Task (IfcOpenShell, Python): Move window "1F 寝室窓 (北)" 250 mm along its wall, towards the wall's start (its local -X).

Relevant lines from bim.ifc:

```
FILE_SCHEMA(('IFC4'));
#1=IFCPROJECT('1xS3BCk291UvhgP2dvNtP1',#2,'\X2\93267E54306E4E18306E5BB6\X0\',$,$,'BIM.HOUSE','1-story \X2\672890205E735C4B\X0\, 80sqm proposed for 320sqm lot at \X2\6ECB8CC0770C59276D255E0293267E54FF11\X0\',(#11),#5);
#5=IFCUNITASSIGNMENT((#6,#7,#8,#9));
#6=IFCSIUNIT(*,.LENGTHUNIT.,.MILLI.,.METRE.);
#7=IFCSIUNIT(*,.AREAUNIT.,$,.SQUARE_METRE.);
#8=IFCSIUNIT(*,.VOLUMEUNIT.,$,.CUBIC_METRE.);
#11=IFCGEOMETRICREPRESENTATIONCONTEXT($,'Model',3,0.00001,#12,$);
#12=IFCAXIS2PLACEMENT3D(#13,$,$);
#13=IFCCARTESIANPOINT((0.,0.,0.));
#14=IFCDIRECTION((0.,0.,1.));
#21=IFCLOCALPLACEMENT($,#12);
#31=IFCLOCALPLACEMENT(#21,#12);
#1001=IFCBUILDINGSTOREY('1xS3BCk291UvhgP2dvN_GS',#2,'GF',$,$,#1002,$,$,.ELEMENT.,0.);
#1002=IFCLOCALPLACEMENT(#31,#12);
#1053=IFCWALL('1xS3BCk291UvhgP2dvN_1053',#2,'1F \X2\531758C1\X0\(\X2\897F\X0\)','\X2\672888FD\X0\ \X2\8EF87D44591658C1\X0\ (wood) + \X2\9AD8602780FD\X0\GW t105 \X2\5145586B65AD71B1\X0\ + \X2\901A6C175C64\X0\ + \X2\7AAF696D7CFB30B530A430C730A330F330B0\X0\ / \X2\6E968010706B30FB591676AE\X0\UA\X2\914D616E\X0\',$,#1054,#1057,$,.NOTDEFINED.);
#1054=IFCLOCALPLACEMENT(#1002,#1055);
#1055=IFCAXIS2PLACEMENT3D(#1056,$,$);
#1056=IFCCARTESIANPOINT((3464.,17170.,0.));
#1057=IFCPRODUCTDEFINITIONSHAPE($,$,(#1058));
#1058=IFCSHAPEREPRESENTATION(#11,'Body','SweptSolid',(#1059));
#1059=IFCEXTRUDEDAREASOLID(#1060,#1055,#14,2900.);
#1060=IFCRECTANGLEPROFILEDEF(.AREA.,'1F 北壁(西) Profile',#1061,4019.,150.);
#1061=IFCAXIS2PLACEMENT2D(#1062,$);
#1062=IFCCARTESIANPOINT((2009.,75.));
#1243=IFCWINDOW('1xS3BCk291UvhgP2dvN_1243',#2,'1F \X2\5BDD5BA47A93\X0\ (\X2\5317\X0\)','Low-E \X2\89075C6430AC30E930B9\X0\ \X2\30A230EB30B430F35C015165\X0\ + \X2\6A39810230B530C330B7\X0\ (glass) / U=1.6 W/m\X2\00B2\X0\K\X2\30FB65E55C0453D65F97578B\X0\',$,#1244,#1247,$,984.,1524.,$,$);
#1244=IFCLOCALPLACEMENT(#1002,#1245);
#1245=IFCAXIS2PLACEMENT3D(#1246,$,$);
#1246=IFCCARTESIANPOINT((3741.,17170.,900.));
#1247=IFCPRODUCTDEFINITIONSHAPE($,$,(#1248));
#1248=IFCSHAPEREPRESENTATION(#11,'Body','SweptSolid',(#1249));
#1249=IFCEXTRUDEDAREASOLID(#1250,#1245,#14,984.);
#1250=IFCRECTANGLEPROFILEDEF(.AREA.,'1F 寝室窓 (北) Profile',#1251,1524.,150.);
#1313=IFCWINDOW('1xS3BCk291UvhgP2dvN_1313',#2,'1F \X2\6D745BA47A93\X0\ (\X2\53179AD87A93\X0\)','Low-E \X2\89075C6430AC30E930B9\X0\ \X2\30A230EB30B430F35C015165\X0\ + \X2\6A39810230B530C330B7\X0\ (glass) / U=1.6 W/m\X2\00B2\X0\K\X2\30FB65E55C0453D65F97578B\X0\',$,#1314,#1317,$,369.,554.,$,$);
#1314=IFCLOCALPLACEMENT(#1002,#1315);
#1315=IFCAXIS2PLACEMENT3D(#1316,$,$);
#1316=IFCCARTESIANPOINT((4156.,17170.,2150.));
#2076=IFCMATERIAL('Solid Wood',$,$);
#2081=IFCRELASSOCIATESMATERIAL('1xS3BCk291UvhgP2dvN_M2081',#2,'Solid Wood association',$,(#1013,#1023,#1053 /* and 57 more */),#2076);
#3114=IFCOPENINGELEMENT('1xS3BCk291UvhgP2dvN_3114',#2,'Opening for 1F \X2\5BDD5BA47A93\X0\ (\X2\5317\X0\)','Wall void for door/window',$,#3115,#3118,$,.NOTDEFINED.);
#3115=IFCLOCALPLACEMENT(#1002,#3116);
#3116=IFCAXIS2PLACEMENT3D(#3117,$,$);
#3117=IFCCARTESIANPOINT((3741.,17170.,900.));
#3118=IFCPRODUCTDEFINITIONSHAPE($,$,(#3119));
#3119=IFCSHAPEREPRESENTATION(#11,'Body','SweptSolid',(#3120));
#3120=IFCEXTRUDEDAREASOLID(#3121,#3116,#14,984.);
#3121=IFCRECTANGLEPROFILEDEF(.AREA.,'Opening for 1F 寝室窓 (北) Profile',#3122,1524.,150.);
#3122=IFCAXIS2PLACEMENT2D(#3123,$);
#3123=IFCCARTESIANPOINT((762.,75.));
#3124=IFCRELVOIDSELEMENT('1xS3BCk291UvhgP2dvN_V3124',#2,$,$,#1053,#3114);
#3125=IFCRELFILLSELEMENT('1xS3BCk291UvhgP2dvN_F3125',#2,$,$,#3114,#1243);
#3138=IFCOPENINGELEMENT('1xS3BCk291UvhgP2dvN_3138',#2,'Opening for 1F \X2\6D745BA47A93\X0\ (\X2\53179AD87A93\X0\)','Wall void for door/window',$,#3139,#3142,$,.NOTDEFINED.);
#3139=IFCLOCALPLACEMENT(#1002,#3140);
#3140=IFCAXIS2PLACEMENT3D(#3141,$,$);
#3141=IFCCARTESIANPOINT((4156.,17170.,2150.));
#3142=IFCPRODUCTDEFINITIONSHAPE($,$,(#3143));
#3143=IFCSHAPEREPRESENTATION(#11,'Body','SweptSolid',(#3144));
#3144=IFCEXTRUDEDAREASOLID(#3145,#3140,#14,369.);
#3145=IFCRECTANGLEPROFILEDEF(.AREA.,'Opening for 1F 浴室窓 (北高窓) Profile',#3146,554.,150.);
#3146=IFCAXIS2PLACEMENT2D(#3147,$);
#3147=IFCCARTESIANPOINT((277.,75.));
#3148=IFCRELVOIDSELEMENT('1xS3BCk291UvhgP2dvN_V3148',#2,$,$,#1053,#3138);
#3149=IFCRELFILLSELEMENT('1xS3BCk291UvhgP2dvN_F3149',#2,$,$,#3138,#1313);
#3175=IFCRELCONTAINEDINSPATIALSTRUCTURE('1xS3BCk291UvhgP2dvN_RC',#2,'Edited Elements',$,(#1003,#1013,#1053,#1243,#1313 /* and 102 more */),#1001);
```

```python
import ifcopenshell
import ifcopenshell.api.geometry
import ifcopenshell.util.placement

model = ifcopenshell.open("bim.ifc")

window = model.by_id(1243)
opening = window.FillsVoids[0].RelatingOpeningElement
wall = opening.VoidsElements[0].RelatingBuildingElement

wall_matrix = ifcopenshell.util.placement.get_local_placement(wall.ObjectPlacement)
shift = wall_matrix[:3, 0] * -250.0
before = ifcopenshell.util.placement.get_local_placement(window.ObjectPlacement)[:3, 3].copy()

# The window is not placed relative to its opening, so move both.
for product in (opening, window):
    matrix = ifcopenshell.util.placement.get_local_placement(product.ObjectPlacement)
    matrix[:3, 3] += shift
    ifcopenshell.api.geometry.edit_object_placement(model, product=product, matrix=matrix, is_si=False)

after = ifcopenshell.util.placement.get_local_placement(window.ObjectPlacement)[:3, 3]
print("window moved by", (after - before).round(3) + 0.0)

model.write("bim_edited.ifc")
```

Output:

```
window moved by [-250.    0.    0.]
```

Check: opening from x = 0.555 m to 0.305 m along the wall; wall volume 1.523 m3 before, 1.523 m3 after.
